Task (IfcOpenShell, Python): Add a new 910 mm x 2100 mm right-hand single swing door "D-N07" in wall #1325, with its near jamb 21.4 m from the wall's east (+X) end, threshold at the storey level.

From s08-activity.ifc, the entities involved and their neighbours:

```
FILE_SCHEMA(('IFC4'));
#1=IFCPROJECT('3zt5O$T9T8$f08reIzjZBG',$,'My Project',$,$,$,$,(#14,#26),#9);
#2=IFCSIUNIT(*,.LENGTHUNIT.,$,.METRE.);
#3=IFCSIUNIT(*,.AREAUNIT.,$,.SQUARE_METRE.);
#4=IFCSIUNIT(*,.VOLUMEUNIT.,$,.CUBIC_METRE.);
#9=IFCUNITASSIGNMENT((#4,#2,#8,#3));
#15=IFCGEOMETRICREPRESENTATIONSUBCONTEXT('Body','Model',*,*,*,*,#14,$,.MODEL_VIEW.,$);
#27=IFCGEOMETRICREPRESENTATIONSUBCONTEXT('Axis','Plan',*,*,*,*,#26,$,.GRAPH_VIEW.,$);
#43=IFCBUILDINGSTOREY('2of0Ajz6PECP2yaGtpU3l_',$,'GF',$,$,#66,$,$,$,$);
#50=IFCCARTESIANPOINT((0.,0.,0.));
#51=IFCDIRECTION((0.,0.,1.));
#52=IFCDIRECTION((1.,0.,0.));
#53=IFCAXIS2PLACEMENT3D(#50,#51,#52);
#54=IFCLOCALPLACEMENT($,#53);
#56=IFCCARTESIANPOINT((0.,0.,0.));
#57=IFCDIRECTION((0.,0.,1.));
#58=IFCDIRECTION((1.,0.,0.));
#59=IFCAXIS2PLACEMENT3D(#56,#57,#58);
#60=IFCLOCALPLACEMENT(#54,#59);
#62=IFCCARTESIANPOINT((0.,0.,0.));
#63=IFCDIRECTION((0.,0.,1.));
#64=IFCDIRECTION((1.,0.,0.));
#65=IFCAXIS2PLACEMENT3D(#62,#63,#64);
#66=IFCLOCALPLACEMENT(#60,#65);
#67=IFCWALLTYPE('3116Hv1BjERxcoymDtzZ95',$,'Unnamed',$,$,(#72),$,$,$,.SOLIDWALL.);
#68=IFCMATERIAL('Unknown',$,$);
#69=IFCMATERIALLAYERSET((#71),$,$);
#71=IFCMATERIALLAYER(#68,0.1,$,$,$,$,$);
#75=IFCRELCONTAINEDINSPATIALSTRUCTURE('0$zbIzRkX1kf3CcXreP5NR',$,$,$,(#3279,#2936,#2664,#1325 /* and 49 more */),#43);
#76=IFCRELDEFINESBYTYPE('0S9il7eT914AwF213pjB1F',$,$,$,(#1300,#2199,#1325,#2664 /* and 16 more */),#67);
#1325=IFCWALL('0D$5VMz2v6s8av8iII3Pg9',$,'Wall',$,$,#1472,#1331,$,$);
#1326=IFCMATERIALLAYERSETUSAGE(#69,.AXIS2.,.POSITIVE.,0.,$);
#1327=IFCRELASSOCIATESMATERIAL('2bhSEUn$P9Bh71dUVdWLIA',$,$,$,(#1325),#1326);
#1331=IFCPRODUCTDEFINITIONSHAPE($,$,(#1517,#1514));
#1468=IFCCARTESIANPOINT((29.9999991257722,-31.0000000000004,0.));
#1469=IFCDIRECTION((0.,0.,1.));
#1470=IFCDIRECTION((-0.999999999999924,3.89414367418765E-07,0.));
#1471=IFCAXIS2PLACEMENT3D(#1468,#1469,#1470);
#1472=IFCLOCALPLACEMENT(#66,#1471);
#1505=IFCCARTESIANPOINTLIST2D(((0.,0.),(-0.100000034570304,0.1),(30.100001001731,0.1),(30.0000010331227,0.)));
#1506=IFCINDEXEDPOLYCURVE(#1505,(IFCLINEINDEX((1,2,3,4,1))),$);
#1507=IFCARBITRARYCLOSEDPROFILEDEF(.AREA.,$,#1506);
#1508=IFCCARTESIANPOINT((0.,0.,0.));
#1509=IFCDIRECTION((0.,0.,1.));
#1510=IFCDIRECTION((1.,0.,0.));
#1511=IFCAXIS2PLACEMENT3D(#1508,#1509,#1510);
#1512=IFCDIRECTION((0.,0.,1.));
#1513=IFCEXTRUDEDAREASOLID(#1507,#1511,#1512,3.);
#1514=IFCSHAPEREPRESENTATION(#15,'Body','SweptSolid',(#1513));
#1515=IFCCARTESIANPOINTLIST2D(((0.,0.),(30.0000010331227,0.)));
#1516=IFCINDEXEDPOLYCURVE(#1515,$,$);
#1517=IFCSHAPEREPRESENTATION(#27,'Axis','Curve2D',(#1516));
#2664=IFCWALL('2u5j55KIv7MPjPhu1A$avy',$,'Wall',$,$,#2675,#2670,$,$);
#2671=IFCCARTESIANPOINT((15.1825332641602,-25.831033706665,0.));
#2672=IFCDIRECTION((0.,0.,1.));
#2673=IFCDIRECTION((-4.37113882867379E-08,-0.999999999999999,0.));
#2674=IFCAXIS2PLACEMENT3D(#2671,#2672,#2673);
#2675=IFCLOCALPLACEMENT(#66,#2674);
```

```python
import numpy as np
import ifcopenshell
import ifcopenshell.api.feature
import ifcopenshell.api.geometry
import ifcopenshell.api.root
import ifcopenshell.api.spatial
import ifcopenshell.geom
import ifcopenshell.util.element
import ifcopenshell.util.placement
import ifcopenshell.util.representation
import ifcopenshell.util.shape
import ifcopenshell.util.unit

model = ifcopenshell.open("s08-activity.ifc")
unit_scale = ifcopenshell.util.unit.calculate_unit_scale(model)
settings = ifcopenshell.geom.settings()


def volume(element):
    """Net volume in cubic metres, openings subtracted."""
    shape = ifcopenshell.geom.create_shape(settings, element)
    return ifcopenshell.util.shape.get_volume(shape.geometry)


wall = model.by_guid("0D$5VMz2v6s8av8iII3Pg9")
storey = ifcopenshell.util.element.get_container(wall, ifc_class="IfcBuildingStorey")
context = ifcopenshell.util.representation.get_context(model, "Model", "Body", "MODEL_VIEW")
before = volume(wall)

width, height, from_end, sill = 0.91, 2.1, 21.4, 0.0  # metres

# The wall runs along its own X axis, and the end named is its -X end.
wall_shape = ifcopenshell.geom.create_shape(settings, wall)
x, y, z = ifcopenshell.util.shape.get_vertices(wall_shape.geometry).T
start = x.min() + from_end
face, thickness = float(y.min()), float(y.max() - y.min())
wall_matrix = ifcopenshell.util.placement.get_local_placement(wall.ObjectPlacement)
level = ifcopenshell.util.placement.get_local_placement(storey.ObjectPlacement)[2, 3]


def in_wall(x, y):
    """Placement at x, y metres in the wall's axes, at sill height."""
    matrix = wall_matrix.copy()
    matrix[:, 3] = wall_matrix @ np.array([x / unit_scale, y / unit_scale, 0.0, 1.0])
    matrix[2, 3] = level + sill / unit_scale
    return matrix


# Opening: a box that overshoots both wall faces by 50 mm.
opening = ifcopenshell.api.root.create_entity(model, ifc_class="IfcOpeningElement", predefined_type="OPENING")
box = ifcopenshell.api.geometry.add_wall_representation(
    model, context=context, length=width, height=height, thickness=thickness + 0.1
)
ifcopenshell.api.geometry.assign_representation(model, product=opening, representation=box)
ifcopenshell.api.geometry.edit_object_placement(model, product=opening, matrix=in_wall(start, face - 0.05), is_si=False)
ifcopenshell.api.feature.add_feature(model, feature=opening, element=wall)

door = ifcopenshell.api.root.create_entity(model, ifc_class="IfcDoor", name="D-N07", predefined_type="DOOR")
door.OverallWidth, door.OverallHeight = width / unit_scale, height / unit_scale
door.OperationType = "SINGLE_SWING_RIGHT"
body = ifcopenshell.api.geometry.add_door_representation(
    model,
    context=context,
    overall_width=door.OverallWidth,
    overall_height=door.OverallHeight,
    operation_type="SINGLE_SWING_RIGHT",
    lining_properties={"LiningDepth": thickness / unit_scale, "ThresholdDepth": thickness / unit_scale},
)
ifcopenshell.api.geometry.assign_representation(model, product=door, representation=body)
ifcopenshell.api.spatial.assign_container(model, products=[door], relating_structure=storey)
ifcopenshell.api.feature.add_filling(model, opening=opening, element=door)

# The lining spans the wall, so the door starts at the wall face.
ifcopenshell.api.geometry.edit_object_placement(model, product=door, matrix=in_wall(start, face), is_si=False)

after = volume(wall)

print(f"wall volume {before:.3f} -> {after:.3f} m3")

model.write("s08-activity_edited.ifc")
```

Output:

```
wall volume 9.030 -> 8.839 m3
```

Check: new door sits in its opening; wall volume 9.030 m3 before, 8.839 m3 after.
